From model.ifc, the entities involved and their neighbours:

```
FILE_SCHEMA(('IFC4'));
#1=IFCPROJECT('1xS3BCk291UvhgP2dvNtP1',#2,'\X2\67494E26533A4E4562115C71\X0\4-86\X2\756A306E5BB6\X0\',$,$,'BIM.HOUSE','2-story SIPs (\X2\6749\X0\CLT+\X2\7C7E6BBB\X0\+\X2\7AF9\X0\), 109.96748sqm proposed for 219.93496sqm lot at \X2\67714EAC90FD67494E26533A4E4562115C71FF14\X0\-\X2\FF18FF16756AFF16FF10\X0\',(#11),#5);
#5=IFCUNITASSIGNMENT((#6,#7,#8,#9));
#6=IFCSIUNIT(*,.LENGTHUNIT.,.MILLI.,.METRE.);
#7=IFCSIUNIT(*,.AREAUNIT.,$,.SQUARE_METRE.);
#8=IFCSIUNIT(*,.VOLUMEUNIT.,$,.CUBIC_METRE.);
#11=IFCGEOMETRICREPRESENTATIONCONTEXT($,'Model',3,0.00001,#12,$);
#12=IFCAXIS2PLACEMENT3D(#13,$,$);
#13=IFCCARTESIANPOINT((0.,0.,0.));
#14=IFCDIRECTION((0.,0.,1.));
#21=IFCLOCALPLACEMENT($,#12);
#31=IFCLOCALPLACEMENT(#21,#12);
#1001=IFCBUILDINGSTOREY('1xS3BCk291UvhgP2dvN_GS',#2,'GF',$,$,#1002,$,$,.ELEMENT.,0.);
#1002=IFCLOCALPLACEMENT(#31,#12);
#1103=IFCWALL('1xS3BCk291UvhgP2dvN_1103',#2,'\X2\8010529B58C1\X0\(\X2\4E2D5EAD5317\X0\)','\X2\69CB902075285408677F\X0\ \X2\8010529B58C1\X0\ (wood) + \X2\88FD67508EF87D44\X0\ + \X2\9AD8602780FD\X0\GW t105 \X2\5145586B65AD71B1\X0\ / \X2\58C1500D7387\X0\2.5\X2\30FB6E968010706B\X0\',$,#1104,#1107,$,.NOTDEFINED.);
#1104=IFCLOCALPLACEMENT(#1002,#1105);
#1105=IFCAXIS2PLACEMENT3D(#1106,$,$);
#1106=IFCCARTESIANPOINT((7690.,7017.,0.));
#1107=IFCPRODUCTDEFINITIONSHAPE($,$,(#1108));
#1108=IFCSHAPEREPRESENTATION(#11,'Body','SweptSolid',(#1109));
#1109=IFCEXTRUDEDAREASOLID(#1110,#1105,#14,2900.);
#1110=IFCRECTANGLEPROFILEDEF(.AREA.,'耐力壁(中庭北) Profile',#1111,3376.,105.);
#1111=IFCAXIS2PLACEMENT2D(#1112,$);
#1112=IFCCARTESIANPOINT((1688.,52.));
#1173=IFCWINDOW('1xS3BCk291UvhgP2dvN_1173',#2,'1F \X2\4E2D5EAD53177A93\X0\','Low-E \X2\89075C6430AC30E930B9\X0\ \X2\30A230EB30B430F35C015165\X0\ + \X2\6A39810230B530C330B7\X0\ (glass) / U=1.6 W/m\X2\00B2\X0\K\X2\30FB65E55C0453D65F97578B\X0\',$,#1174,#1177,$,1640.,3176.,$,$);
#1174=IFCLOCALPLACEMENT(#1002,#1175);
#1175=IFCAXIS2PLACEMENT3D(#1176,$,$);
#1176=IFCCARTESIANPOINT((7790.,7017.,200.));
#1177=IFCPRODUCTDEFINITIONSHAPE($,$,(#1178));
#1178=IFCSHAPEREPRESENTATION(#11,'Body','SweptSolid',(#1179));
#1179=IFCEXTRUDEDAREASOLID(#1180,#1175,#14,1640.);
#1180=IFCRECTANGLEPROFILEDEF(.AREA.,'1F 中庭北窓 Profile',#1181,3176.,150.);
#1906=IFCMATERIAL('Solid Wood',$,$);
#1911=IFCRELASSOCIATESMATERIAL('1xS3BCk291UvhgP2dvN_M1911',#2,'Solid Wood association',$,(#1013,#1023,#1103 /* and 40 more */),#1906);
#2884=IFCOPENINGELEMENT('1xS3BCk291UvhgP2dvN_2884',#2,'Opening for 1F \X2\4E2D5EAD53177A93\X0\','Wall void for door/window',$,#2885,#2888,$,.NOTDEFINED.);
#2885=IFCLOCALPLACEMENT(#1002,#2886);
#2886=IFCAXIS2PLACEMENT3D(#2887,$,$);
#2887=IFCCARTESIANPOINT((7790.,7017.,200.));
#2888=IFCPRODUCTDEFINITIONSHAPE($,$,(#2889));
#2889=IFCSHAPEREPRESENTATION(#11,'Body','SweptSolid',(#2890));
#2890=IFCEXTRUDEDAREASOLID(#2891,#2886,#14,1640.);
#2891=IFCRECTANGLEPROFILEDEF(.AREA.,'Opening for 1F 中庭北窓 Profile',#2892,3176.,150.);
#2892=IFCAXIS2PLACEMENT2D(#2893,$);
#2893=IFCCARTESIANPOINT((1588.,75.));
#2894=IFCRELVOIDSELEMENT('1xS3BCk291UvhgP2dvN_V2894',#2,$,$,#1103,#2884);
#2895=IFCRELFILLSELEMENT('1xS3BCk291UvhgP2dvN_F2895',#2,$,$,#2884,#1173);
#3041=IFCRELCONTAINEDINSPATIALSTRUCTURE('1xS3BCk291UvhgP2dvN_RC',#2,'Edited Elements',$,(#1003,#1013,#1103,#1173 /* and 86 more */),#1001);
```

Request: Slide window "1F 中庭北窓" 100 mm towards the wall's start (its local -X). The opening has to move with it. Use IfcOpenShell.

```python
import ifcopenshell
import ifcopenshell.api.geometry
import ifcopenshell.util.placement
import ifcopenshell.util.unit

model = ifcopenshell.open("model.ifc")
unit_scale = ifcopenshell.util.unit.calculate_unit_scale(model)

window = model.by_guid("1xS3BCk291UvhgP2dvN_1173")
opening = window.FillsVoids[0].RelatingOpeningElement
wall = opening.VoidsElements[0].RelatingBuildingElement

wall_matrix = ifcopenshell.util.placement.get_local_placement(wall.ObjectPlacement)
shift = wall_matrix[:3, 0] * -0.1 / unit_scale
before = ifcopenshell.util.placement.get_local_placement(window.ObjectPlacement)[:3, 3].copy()

# The window is not placed relative to its opening, so move both.
for product in (opening, window):
    matrix = ifcopenshell.util.placement.get_local_placement(product.ObjectPlacement)
    matrix[:3, 3] += shift
    ifcopenshell.api.geometry.edit_object_placement(model, product=product, matrix=matrix, is_si=False)

after = ifcopenshell.util.placement.get_local_placement(window.ObjectPlacement)[:3, 3]
print("window moved by", (after - before).round(3) + 0.0)

model.write("model_updated.ifc")
```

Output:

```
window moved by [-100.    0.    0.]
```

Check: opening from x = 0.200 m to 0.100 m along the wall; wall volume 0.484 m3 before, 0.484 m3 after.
